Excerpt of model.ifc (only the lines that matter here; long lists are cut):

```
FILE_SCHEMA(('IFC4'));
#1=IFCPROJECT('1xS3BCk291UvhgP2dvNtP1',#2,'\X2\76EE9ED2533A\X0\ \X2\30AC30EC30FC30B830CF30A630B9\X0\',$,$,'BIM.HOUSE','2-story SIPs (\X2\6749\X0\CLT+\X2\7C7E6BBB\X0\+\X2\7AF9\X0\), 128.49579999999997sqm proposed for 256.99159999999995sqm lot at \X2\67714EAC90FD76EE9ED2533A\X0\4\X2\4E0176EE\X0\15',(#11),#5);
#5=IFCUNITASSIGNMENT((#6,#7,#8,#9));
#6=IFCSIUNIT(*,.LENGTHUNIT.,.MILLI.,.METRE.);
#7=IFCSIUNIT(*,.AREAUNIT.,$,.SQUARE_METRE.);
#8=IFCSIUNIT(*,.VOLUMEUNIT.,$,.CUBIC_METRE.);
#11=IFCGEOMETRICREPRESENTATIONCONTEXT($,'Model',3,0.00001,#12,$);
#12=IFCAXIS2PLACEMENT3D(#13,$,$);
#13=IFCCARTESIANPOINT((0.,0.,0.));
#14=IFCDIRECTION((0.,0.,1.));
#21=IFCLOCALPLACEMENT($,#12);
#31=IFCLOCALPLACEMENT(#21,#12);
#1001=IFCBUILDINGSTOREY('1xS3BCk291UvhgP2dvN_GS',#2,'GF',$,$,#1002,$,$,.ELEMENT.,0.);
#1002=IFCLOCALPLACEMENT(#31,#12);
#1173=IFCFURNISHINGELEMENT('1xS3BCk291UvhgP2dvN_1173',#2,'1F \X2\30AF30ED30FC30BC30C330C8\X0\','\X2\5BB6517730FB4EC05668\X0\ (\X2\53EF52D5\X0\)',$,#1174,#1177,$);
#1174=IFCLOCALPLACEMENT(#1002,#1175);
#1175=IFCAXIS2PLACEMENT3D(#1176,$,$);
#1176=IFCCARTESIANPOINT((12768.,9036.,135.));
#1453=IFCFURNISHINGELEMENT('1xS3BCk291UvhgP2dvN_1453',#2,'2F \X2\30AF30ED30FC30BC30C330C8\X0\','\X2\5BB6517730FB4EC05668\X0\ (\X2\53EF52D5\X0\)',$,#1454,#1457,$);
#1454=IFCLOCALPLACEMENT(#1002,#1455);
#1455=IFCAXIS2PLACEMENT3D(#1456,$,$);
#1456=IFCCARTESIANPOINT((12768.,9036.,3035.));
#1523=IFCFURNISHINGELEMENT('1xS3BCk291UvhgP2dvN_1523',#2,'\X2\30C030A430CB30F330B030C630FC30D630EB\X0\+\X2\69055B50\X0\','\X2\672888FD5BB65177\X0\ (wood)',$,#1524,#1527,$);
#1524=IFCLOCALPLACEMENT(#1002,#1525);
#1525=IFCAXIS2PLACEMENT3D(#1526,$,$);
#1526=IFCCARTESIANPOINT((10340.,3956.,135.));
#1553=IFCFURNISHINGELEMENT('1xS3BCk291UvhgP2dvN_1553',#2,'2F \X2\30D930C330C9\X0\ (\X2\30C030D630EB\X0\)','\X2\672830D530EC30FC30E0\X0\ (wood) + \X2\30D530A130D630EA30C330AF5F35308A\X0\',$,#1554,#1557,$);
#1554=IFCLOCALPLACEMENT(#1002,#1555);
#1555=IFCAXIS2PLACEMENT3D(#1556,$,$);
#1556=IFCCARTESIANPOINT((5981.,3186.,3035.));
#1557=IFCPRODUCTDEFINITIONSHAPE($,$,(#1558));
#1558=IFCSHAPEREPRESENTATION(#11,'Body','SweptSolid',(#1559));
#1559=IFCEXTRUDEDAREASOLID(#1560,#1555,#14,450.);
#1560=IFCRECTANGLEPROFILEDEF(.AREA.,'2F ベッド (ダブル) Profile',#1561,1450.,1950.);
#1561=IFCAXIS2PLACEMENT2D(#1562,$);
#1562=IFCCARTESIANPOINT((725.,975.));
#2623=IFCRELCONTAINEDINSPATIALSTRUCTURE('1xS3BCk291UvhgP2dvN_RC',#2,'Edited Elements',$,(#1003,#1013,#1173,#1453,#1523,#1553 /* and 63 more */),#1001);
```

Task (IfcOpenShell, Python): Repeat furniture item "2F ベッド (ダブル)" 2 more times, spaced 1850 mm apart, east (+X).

```python
import numpy as np
import ifcopenshell
import ifcopenshell.api.geometry
import ifcopenshell.api.root
import ifcopenshell.util.element
import ifcopenshell.util.placement
import ifcopenshell.util.unit

model = ifcopenshell.open("model.ifc")
unit_scale = ifcopenshell.util.unit.calculate_unit_scale(model)


def reuse_history(source, copy):
    """copy_class also copies each property set's owner history, people and application; keep the originals."""
    for rel in copy.IsDefinedBy:
        if rel.is_a("IfcRelDefinesByProperties") and (history := rel.RelatingPropertyDefinition.OwnerHistory):
            rel.RelatingPropertyDefinition.OwnerHistory = source.OwnerHistory
            ifcopenshell.util.element.remove_deep2(model, history)


source = model.by_guid("1xS3BCk291UvhgP2dvN_1553")
base = ifcopenshell.util.placement.get_local_placement(source.ObjectPlacement)
step = np.array([1.0, 0.0, 0.0]) * 1.85 / unit_scale

for i in range(1, 3):
    copy = ifcopenshell.api.root.copy_class(model, product=source)
    copy.Representation = ifcopenshell.util.element.copy_deep(
        model, source.Representation, exclude=["IfcGeometricRepresentationContext", "IfcRepresentationMap"]
    )
    reuse_history(source, copy)
    matrix = base.copy()
    matrix[:3, 3] += i * step
    print("added at", matrix[:3, 3].round(3) + 0.0)
    ifcopenshell.api.geometry.edit_object_placement(model, product=copy, matrix=matrix, is_si=False)

model.write("model_v2.ifc")
```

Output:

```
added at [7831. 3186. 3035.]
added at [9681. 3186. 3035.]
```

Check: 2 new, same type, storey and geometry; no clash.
